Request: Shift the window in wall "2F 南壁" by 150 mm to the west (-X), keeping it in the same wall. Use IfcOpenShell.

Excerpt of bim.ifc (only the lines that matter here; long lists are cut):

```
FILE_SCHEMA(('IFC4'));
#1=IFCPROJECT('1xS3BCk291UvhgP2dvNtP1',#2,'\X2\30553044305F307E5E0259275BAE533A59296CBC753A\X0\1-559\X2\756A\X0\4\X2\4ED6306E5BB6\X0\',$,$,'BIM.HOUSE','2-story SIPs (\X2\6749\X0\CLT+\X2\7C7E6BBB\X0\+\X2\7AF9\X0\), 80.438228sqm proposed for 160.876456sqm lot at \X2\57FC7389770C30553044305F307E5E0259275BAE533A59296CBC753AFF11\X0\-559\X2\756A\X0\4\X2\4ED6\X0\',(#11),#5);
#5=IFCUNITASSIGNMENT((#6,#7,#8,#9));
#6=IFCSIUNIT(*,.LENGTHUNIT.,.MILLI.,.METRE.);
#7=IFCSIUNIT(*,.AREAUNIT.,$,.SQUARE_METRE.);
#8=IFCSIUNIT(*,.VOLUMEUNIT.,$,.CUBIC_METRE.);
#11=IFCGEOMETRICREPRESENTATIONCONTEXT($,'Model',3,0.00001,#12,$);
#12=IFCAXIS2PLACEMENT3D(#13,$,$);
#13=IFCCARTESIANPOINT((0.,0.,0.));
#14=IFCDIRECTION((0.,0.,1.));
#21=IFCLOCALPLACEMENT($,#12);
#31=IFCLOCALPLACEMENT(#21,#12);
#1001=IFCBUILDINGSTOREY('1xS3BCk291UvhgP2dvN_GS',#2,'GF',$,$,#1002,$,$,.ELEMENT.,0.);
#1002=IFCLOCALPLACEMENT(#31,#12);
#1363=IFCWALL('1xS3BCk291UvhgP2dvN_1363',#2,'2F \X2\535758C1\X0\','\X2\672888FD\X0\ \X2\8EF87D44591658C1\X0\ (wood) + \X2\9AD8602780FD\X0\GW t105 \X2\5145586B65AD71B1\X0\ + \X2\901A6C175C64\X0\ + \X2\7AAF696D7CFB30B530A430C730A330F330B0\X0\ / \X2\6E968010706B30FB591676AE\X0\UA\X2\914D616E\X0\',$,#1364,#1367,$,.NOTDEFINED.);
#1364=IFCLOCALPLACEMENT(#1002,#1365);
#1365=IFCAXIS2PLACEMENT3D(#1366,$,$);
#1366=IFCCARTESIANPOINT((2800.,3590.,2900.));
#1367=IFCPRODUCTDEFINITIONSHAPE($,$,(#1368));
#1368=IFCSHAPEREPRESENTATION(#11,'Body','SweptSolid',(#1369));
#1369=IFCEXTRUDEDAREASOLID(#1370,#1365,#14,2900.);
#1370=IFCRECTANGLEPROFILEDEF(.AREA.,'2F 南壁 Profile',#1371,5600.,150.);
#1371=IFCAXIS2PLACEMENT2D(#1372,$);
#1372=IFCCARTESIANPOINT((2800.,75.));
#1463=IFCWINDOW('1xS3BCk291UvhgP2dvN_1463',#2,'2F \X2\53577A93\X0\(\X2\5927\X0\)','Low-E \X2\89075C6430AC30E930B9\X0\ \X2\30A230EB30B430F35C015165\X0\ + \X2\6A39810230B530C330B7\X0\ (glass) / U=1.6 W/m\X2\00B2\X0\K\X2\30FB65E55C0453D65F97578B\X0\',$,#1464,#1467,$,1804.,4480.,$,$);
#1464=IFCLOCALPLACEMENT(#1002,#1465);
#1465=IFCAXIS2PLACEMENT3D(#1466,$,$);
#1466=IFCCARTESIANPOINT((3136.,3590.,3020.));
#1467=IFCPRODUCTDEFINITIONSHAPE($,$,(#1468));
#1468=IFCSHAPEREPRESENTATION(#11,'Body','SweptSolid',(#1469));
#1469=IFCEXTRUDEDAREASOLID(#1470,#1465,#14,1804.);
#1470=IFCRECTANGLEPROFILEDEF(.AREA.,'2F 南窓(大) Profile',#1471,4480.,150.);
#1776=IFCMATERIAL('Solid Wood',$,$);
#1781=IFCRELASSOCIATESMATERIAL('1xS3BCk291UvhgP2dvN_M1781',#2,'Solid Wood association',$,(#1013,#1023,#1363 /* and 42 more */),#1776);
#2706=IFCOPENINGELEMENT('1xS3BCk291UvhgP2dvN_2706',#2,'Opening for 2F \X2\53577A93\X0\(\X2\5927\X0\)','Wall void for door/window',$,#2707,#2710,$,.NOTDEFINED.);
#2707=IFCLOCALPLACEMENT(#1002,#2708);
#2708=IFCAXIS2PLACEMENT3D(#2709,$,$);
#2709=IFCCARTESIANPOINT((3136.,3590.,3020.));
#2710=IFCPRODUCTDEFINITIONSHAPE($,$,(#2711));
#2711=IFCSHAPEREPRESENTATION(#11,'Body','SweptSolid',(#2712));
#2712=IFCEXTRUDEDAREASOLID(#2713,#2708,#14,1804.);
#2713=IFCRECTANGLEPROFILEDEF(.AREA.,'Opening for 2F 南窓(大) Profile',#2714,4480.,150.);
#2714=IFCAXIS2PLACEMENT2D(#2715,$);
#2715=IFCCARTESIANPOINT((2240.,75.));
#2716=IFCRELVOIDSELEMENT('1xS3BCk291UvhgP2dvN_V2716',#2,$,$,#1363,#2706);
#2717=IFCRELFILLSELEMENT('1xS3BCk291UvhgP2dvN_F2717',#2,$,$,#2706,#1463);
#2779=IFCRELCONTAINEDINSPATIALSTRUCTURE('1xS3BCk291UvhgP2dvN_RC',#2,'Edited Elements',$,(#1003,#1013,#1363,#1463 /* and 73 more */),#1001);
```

```python
import ifcopenshell
import ifcopenshell.api.geometry
import ifcopenshell.util.placement
import ifcopenshell.util.unit

model = ifcopenshell.open("bim.ifc")
unit_scale = ifcopenshell.util.unit.calculate_unit_scale(model)

window = model.by_guid("1xS3BCk291UvhgP2dvN_1463")
opening = window.FillsVoids[0].RelatingOpeningElement
wall = opening.VoidsElements[0].RelatingBuildingElement

wall_matrix = ifcopenshell.util.placement.get_local_placement(wall.ObjectPlacement)
shift = wall_matrix[:3, 0] * -0.15 / unit_scale
before = ifcopenshell.util.placement.get_local_placement(window.ObjectPlacement)[:3, 3].copy()

# The window is not placed relative to its opening, so move both.
for product in (opening, window):
    matrix = ifcopenshell.util.placement.get_local_placement(product.ObjectPlacement)
    matrix[:3, 3] += shift
    ifcopenshell.api.geometry.edit_object_placement(model, product=product, matrix=matrix, is_si=False)

after = ifcopenshell.util.placement.get_local_placement(window.ObjectPlacement)[:3, 3]
print("window moved by", (after - before).round(3) + 0.0)

model.write("bim-out.ifc")
```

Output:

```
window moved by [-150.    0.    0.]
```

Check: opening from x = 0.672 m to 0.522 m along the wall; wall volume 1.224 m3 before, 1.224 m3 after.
